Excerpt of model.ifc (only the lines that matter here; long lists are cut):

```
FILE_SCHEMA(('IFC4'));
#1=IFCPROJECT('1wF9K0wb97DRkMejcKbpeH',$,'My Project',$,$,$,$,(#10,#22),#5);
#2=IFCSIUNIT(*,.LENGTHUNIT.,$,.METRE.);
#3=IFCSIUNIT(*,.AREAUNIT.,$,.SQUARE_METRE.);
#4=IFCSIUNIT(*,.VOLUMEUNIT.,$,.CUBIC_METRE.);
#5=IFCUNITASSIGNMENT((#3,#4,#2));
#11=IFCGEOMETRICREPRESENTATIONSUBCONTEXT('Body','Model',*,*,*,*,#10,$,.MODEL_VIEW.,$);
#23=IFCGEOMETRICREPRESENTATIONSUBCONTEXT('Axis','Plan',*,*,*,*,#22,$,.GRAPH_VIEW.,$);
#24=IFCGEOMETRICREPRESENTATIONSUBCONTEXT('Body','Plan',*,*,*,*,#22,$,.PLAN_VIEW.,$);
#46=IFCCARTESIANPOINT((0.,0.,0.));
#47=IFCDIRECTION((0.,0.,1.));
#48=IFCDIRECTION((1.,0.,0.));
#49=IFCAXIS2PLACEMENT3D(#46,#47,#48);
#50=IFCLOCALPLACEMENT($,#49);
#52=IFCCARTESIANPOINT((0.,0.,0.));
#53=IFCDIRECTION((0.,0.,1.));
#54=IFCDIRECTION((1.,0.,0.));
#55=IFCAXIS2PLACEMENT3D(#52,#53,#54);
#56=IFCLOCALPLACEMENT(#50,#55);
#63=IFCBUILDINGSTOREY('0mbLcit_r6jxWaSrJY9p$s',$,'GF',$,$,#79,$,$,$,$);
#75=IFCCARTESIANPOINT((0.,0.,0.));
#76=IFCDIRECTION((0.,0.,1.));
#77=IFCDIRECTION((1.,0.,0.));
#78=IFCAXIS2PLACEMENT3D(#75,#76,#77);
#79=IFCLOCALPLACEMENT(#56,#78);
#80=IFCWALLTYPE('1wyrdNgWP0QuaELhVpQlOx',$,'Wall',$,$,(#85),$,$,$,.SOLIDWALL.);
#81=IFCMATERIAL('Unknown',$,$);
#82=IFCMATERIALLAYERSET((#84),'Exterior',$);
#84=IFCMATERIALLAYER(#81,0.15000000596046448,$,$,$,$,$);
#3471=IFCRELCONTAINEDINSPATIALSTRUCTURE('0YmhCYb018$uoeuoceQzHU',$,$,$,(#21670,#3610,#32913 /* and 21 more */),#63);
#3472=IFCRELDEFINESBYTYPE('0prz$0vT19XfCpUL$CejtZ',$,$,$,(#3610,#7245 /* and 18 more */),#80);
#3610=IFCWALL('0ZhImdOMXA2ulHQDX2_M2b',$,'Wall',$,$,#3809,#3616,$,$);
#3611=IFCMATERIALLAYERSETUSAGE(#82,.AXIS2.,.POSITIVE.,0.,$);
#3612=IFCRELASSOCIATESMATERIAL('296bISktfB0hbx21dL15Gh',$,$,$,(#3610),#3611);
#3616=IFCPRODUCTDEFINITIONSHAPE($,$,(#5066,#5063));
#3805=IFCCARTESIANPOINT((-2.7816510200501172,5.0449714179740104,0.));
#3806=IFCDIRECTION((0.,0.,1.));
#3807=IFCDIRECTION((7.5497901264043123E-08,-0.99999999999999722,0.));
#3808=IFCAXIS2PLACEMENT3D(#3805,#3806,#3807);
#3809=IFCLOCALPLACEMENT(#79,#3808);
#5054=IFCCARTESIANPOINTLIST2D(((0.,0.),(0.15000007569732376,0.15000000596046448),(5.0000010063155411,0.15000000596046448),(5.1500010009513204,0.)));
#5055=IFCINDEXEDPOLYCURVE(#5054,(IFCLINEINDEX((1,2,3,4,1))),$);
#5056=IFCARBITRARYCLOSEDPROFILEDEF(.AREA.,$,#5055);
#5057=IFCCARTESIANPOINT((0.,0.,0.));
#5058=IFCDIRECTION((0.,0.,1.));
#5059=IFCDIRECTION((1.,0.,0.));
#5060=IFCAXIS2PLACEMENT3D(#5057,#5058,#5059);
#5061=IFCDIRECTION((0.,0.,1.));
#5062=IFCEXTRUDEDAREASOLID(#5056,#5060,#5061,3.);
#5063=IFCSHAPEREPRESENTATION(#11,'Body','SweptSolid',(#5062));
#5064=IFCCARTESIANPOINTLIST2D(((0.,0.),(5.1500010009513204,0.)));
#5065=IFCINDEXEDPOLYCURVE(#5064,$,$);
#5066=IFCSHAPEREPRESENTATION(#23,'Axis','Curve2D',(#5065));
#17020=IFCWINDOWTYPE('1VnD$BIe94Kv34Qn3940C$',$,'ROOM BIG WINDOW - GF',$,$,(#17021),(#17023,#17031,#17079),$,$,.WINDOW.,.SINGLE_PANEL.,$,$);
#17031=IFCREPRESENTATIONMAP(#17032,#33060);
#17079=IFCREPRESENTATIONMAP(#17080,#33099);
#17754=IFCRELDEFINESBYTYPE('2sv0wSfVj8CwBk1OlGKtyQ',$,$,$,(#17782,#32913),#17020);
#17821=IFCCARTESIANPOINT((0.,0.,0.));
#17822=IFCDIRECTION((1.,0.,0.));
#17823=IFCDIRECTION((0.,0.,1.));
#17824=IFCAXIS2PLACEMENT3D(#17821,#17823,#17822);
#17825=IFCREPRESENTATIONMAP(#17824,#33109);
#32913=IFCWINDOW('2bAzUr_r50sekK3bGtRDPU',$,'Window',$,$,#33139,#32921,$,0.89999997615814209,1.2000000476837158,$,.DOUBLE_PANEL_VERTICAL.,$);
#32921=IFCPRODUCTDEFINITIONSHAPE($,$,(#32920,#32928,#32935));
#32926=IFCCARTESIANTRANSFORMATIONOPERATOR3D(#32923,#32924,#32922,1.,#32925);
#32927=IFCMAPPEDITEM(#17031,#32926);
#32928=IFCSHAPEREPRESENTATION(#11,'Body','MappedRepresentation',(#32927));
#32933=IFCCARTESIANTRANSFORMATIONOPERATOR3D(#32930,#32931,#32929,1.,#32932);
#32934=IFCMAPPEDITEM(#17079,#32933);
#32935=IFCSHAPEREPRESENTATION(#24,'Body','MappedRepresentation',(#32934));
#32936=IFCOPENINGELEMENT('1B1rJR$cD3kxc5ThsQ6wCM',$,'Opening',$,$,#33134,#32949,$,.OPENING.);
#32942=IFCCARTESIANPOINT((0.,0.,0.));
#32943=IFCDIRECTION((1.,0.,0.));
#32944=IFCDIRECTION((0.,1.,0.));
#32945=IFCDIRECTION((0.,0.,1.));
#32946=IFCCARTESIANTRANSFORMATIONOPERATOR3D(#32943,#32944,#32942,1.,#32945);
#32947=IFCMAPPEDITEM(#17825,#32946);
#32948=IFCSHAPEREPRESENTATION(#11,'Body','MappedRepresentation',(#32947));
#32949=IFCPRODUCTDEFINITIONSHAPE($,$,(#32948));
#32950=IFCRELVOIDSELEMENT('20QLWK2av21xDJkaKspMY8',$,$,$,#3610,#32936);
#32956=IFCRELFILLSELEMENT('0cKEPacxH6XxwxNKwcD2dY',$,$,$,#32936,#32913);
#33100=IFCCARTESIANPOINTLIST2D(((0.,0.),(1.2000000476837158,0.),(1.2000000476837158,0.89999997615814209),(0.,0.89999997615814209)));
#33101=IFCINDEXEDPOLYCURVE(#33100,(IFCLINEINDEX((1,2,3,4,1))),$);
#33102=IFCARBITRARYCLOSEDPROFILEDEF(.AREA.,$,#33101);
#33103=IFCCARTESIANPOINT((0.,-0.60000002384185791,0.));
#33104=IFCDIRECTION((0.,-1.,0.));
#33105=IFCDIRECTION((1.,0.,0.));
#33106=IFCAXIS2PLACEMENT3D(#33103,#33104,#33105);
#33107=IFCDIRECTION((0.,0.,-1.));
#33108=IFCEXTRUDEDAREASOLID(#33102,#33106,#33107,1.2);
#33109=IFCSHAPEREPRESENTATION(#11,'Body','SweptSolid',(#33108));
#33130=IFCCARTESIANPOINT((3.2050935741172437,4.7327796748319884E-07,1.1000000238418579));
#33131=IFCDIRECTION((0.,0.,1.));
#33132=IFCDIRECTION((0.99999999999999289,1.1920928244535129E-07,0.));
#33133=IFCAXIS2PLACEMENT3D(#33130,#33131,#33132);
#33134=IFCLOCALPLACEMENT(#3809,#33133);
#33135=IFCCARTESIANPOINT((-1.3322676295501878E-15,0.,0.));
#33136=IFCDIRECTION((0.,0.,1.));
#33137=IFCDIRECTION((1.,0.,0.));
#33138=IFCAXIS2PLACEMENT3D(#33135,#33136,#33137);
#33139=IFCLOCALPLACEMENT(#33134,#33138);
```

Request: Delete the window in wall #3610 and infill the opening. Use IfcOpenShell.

```python
import ifcopenshell
import ifcopenshell.api.feature
import ifcopenshell.api.root
import ifcopenshell.geom
import ifcopenshell.util.shape

model = ifcopenshell.open("model.ifc")
settings = ifcopenshell.geom.settings()


def volume(element):
    """Net volume in cubic metres, openings subtracted."""
    shape = ifcopenshell.geom.create_shape(settings, element)
    return ifcopenshell.util.shape.get_volume(shape.geometry)


window = model.by_guid("2bAzUr_r50sekK3bGtRDPU")
opening = window.FillsVoids[0].RelatingOpeningElement
wall = opening.VoidsElements[0].RelatingBuildingElement
before = volume(wall)

ifcopenshell.api.root.remove_product(model, product=window)
ifcopenshell.api.feature.remove_feature(model, feature=opening)

after = volume(wall)

print(f"wall volume {before:.3f} -> {after:.3f} m3")

model.write("model_edited.ifc")
```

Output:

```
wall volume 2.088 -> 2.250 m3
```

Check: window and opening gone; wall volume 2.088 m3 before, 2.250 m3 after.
